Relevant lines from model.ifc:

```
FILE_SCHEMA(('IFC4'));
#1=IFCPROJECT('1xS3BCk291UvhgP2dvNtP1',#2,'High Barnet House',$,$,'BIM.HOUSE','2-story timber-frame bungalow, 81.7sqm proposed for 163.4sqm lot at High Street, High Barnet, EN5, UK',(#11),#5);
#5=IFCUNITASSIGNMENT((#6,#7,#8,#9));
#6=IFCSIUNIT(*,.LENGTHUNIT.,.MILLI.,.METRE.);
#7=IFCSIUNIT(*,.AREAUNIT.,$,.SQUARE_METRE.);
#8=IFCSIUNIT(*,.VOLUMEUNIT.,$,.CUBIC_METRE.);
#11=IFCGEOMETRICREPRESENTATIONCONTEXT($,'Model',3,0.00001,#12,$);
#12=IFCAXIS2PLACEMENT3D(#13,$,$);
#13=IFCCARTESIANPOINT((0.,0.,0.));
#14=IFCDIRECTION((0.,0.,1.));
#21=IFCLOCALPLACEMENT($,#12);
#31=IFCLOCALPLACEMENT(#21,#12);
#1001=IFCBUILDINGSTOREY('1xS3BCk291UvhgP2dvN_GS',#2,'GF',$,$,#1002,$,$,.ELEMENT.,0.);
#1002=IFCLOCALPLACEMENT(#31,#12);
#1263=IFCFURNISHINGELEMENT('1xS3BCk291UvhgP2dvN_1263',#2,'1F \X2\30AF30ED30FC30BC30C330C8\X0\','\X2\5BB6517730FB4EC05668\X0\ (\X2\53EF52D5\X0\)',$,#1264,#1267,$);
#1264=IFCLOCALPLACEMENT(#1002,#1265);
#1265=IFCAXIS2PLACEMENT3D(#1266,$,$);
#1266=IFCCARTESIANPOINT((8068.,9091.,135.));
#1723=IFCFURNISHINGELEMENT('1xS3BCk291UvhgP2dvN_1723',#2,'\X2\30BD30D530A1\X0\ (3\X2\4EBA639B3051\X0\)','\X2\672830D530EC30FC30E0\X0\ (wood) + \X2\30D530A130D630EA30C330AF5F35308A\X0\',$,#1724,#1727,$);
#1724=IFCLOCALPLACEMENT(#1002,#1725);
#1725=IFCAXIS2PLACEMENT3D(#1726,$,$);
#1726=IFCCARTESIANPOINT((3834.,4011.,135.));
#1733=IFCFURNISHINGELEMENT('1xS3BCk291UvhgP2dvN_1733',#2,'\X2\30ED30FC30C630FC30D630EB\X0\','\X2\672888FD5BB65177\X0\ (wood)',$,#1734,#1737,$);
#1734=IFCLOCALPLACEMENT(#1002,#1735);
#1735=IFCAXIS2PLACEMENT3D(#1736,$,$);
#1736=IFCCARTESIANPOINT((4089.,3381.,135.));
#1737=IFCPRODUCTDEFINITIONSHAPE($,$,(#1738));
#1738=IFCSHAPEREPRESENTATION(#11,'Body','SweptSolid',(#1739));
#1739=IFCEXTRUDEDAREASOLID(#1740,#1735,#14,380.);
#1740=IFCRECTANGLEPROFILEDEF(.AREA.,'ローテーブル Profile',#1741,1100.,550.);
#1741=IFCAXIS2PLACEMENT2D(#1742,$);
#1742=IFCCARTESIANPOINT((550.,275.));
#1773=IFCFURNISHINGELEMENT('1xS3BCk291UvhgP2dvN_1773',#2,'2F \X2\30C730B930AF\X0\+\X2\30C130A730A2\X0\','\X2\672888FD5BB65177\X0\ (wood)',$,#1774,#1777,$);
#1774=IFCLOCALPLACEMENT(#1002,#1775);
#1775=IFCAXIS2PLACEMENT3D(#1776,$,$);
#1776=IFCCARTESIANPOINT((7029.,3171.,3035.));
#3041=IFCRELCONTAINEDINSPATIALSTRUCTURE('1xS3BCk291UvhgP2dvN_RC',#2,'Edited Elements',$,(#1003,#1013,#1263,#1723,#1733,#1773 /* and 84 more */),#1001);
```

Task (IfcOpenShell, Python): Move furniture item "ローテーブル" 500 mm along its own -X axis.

```python
import ifcopenshell
import ifcopenshell.api.geometry
import ifcopenshell.util.placement

model = ifcopenshell.open("model.ifc")

item = model.by_id(1733)
matrix = ifcopenshell.util.placement.get_local_placement(item.ObjectPlacement)
matrix[:3, 3] -= matrix[:3, 0] * 500.0
ifcopenshell.api.geometry.edit_object_placement(model, product=item, matrix=matrix, is_si=False)

print(ifcopenshell.util.placement.get_local_placement(item.ObjectPlacement).round(3) + 0.0)

model.write("model_rev.ifc")
```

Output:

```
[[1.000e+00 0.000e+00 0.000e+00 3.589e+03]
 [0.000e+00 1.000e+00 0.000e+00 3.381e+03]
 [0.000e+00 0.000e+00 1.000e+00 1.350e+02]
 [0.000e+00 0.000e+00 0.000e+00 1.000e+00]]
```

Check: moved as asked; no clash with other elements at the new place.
